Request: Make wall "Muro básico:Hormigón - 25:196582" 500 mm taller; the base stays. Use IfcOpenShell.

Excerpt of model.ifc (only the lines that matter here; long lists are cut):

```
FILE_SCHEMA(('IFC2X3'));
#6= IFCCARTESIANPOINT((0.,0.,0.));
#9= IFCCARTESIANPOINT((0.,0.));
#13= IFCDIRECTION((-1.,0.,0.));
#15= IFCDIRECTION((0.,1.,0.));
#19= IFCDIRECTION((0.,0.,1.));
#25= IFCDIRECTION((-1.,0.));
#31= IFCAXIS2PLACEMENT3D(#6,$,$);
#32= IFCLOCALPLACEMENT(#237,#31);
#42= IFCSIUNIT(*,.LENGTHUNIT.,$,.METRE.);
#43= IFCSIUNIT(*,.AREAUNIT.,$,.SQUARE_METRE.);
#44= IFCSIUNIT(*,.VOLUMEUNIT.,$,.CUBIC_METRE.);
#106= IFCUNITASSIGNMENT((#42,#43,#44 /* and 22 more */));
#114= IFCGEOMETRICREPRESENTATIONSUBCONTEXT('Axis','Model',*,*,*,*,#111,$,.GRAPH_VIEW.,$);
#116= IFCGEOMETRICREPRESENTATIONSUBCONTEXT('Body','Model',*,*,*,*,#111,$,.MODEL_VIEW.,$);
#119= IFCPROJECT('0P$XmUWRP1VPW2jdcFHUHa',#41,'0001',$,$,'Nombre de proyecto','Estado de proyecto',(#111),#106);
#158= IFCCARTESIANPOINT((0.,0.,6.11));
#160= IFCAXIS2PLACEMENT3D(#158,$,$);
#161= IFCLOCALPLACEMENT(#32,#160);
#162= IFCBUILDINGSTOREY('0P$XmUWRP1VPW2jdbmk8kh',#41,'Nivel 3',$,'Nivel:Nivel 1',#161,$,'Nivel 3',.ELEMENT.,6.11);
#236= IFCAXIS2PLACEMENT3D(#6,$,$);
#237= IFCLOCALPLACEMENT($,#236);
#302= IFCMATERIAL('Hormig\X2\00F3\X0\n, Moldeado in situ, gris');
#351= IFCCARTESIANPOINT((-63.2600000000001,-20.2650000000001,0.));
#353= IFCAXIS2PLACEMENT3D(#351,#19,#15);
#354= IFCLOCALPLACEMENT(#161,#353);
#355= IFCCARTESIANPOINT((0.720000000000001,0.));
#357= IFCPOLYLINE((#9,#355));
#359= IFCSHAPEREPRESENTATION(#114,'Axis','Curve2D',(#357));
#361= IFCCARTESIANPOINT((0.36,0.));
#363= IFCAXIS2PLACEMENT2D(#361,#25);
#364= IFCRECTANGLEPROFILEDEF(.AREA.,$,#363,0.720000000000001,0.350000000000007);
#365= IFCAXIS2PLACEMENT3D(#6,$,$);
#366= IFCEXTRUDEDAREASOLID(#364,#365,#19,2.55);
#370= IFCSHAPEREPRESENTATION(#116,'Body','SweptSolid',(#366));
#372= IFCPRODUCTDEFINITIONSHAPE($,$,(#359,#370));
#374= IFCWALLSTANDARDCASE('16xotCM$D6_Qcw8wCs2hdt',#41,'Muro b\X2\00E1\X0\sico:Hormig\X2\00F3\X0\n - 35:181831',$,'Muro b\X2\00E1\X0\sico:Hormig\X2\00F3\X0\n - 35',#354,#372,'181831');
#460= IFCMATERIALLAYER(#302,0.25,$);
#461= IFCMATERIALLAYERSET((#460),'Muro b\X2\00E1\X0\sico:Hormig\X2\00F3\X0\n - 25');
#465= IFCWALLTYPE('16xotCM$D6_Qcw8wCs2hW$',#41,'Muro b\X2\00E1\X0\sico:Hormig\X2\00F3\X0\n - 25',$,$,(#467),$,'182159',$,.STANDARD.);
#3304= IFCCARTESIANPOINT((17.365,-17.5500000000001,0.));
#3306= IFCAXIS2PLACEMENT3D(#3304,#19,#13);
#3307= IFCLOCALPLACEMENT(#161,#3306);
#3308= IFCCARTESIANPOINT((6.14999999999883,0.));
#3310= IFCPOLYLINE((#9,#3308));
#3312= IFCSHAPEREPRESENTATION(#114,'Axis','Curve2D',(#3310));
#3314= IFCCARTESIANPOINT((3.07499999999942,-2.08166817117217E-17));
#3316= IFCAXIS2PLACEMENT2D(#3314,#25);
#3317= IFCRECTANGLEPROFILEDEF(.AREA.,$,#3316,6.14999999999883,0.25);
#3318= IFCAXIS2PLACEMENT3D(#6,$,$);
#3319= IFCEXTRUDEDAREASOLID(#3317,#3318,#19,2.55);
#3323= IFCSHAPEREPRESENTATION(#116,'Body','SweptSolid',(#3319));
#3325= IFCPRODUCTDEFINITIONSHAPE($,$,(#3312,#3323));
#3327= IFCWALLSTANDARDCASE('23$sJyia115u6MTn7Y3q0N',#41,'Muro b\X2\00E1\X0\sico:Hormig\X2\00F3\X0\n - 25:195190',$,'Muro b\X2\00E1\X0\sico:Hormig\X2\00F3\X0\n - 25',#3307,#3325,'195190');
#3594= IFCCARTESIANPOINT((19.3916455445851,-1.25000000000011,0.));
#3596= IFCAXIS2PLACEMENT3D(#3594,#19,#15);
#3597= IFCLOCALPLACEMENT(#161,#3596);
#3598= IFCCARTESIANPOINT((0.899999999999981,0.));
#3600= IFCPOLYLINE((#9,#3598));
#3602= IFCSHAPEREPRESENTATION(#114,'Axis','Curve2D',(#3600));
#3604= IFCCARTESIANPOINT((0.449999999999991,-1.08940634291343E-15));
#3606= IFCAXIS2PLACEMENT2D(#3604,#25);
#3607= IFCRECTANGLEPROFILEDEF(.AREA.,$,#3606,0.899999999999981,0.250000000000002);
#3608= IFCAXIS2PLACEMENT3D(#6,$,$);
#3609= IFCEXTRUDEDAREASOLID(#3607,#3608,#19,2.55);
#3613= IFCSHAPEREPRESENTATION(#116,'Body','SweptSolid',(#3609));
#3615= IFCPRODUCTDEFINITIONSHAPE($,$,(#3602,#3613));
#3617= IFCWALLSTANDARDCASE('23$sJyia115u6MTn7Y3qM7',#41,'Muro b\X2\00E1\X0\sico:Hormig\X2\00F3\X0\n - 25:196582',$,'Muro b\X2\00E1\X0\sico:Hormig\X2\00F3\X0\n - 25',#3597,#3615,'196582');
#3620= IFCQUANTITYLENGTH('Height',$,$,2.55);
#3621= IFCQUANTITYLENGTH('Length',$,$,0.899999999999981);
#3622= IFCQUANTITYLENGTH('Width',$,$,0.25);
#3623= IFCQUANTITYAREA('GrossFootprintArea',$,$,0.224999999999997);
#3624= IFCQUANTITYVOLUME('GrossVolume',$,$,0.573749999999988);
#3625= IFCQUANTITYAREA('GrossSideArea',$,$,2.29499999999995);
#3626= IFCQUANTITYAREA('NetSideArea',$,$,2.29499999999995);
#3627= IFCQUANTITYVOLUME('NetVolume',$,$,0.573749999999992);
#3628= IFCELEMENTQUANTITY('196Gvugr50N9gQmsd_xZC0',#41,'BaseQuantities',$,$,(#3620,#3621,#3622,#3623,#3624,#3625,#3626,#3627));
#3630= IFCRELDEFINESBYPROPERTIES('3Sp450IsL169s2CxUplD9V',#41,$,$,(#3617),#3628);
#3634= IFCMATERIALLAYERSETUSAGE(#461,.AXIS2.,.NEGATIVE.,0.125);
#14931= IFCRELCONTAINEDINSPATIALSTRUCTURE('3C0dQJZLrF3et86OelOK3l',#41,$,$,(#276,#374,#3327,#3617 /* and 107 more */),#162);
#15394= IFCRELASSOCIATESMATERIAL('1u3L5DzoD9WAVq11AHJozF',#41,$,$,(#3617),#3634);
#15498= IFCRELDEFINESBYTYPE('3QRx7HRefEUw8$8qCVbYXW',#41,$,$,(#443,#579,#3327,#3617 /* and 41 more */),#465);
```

```python
import ifcopenshell
import ifcopenshell.api.pset
import ifcopenshell.geom
import ifcopenshell.util.element
import ifcopenshell.util.representation
import ifcopenshell.util.shape
import ifcopenshell.util.unit

model = ifcopenshell.open("model.ifc")
unit_scale = ifcopenshell.util.unit.calculate_unit_scale(model)
area_scale = ifcopenshell.util.unit.calculate_unit_scale(model, "AREAUNIT")
volume_scale = ifcopenshell.util.unit.calculate_unit_scale(model, "VOLUMEUNIT")
settings = ifcopenshell.geom.settings()


def volume(element):
    """Net volume in cubic metres, openings subtracted."""
    shape = ifcopenshell.geom.create_shape(settings, element)
    return ifcopenshell.util.shape.get_volume(shape.geometry)


wall = model.by_guid("23$sJyia115u6MTn7Y3qM7")
before = volume(wall)

body = ifcopenshell.util.representation.get_representation(wall, "Model", "Body")
solid = body.Items[0]
old_height = solid.Depth
solid.Depth += 0.5
after = volume(wall)
thickness = 0.25  # wall thickness in metres

# Update the stored height, areas and volumes.
qto = model.by_id(ifcopenshell.util.element.get_pset(wall, "BaseQuantities", should_inherit=False)["id"])
ifcopenshell.api.pset.edit_qto(model, qto=qto, properties={
    "Height": solid.Depth,
    "GrossVolume": ifcopenshell.util.element.get_pset(wall, "BaseQuantities", "GrossVolume") * solid.Depth / old_height,
    "GrossSideArea": ifcopenshell.util.element.get_pset(wall, "BaseQuantities", "GrossSideArea") * solid.Depth / old_height,
    "NetSideArea": after / thickness / area_scale,
    "NetVolume": after / volume_scale,
})

print(f"height {old_height:g} -> {solid.Depth:g}, volume {before:.3f} -> {after:.3f} m3")

model.write("model_edited.ifc")
```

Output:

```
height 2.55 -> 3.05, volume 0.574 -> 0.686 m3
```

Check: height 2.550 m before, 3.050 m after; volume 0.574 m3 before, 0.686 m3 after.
